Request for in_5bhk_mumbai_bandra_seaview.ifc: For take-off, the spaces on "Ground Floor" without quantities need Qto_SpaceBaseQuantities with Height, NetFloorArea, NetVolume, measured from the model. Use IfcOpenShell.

First a look at what the model holds.

```python
import ifcopenshell
import ifcopenshell.util.element
import ifcopenshell.util.unit

model = ifcopenshell.open("in_5bhk_mumbai_bandra_seaview.ifc")
print(model.schema)
for unit_type in ("LENGTHUNIT", "AREAUNIT", "VOLUMEUNIT"):
    print(unit_type, ifcopenshell.util.unit.calculate_unit_scale(model, unit_type))
storey = next(s for s in model.by_type("IfcBuildingStorey") if s.Name == "Ground Floor")
spaces = [e for e in ifcopenshell.util.element.get_decomposition(storey) if e.is_a("IfcSpace")]
for e in sorted(spaces, key=lambda e: e.id()):
    print(e.id(), e.is_a(), e.Name, list(ifcopenshell.util.element.get_psets(e, qtos_only=True)), sep=" | ")
```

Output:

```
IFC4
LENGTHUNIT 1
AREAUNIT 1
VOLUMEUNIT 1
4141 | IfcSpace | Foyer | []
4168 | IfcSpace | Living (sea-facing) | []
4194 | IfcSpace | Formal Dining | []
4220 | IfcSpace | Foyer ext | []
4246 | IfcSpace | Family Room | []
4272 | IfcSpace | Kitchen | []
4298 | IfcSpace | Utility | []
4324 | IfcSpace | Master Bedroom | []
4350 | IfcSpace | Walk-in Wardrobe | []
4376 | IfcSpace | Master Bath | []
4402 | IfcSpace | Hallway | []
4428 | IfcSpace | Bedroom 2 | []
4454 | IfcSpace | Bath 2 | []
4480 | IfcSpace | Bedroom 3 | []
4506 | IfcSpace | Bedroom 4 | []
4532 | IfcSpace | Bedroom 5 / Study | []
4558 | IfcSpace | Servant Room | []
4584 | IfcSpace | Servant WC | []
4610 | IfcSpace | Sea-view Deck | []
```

```python
import ifcopenshell
import ifcopenshell.api.pset
import ifcopenshell.geom
import ifcopenshell.util.element
import ifcopenshell.util.shape
import ifcopenshell.util.unit

model = ifcopenshell.open("in_5bhk_mumbai_bandra_seaview.ifc")
unit_scale = ifcopenshell.util.unit.calculate_unit_scale(model)
area_scale = ifcopenshell.util.unit.calculate_unit_scale(model, "AREAUNIT")
volume_scale = ifcopenshell.util.unit.calculate_unit_scale(model, "VOLUMEUNIT")
settings = ifcopenshell.geom.settings()

storey = next(s for s in model.by_type("IfcBuildingStorey") if s.Name == "Ground Floor")
spaces = [e for e in ifcopenshell.util.element.get_decomposition(storey) if e.is_a("IfcSpace")]

for e in sorted(spaces, key=lambda e: e.id()):
    if ifcopenshell.util.element.get_psets(e, qtos_only=True, should_inherit=False):
        continue
    # Geometry comes back in metres, in the element's own axes.
    shape = ifcopenshell.geom.create_shape(settings, e)
    values = {
        "Height": ifcopenshell.util.shape.get_z(shape.geometry) / unit_scale,
        "NetFloorArea": ifcopenshell.util.shape.get_footprint_area(shape.geometry) / area_scale,
        "NetVolume": ifcopenshell.util.shape.get_volume(shape.geometry) / volume_scale,
    }
    qto = ifcopenshell.api.pset.add_qto(model, product=e, name="Qto_SpaceBaseQuantities")
    ifcopenshell.api.pset.edit_qto(model, qto=qto, properties=values)
    print(e.id(), {k: round(v, 3) for k, v in values.items()})

model.write("in_5bhk_mumbai_bandra_seaview_edited.ifc")
```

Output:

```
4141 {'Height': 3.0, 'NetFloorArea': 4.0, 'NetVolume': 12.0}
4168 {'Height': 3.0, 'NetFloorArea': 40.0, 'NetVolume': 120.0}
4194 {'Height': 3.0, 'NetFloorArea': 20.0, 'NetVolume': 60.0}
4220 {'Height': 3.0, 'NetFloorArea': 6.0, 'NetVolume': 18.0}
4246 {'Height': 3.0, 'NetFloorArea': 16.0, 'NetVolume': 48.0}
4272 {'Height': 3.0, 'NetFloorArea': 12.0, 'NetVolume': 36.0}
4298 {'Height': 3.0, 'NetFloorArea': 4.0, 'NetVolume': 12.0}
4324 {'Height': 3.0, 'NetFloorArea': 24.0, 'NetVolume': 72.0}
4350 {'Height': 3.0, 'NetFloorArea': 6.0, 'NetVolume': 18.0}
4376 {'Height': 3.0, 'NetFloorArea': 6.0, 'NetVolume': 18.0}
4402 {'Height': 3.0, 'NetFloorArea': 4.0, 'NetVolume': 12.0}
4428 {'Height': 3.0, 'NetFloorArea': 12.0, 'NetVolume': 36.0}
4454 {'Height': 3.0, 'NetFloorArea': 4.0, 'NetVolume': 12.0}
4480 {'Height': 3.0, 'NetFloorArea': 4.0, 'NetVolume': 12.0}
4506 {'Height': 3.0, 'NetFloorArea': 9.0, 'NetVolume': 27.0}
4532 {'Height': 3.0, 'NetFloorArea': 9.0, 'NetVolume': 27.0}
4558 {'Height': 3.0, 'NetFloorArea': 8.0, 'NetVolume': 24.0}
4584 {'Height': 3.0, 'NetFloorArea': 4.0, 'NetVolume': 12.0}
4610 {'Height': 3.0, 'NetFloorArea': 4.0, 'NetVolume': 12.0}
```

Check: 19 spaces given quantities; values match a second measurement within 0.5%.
